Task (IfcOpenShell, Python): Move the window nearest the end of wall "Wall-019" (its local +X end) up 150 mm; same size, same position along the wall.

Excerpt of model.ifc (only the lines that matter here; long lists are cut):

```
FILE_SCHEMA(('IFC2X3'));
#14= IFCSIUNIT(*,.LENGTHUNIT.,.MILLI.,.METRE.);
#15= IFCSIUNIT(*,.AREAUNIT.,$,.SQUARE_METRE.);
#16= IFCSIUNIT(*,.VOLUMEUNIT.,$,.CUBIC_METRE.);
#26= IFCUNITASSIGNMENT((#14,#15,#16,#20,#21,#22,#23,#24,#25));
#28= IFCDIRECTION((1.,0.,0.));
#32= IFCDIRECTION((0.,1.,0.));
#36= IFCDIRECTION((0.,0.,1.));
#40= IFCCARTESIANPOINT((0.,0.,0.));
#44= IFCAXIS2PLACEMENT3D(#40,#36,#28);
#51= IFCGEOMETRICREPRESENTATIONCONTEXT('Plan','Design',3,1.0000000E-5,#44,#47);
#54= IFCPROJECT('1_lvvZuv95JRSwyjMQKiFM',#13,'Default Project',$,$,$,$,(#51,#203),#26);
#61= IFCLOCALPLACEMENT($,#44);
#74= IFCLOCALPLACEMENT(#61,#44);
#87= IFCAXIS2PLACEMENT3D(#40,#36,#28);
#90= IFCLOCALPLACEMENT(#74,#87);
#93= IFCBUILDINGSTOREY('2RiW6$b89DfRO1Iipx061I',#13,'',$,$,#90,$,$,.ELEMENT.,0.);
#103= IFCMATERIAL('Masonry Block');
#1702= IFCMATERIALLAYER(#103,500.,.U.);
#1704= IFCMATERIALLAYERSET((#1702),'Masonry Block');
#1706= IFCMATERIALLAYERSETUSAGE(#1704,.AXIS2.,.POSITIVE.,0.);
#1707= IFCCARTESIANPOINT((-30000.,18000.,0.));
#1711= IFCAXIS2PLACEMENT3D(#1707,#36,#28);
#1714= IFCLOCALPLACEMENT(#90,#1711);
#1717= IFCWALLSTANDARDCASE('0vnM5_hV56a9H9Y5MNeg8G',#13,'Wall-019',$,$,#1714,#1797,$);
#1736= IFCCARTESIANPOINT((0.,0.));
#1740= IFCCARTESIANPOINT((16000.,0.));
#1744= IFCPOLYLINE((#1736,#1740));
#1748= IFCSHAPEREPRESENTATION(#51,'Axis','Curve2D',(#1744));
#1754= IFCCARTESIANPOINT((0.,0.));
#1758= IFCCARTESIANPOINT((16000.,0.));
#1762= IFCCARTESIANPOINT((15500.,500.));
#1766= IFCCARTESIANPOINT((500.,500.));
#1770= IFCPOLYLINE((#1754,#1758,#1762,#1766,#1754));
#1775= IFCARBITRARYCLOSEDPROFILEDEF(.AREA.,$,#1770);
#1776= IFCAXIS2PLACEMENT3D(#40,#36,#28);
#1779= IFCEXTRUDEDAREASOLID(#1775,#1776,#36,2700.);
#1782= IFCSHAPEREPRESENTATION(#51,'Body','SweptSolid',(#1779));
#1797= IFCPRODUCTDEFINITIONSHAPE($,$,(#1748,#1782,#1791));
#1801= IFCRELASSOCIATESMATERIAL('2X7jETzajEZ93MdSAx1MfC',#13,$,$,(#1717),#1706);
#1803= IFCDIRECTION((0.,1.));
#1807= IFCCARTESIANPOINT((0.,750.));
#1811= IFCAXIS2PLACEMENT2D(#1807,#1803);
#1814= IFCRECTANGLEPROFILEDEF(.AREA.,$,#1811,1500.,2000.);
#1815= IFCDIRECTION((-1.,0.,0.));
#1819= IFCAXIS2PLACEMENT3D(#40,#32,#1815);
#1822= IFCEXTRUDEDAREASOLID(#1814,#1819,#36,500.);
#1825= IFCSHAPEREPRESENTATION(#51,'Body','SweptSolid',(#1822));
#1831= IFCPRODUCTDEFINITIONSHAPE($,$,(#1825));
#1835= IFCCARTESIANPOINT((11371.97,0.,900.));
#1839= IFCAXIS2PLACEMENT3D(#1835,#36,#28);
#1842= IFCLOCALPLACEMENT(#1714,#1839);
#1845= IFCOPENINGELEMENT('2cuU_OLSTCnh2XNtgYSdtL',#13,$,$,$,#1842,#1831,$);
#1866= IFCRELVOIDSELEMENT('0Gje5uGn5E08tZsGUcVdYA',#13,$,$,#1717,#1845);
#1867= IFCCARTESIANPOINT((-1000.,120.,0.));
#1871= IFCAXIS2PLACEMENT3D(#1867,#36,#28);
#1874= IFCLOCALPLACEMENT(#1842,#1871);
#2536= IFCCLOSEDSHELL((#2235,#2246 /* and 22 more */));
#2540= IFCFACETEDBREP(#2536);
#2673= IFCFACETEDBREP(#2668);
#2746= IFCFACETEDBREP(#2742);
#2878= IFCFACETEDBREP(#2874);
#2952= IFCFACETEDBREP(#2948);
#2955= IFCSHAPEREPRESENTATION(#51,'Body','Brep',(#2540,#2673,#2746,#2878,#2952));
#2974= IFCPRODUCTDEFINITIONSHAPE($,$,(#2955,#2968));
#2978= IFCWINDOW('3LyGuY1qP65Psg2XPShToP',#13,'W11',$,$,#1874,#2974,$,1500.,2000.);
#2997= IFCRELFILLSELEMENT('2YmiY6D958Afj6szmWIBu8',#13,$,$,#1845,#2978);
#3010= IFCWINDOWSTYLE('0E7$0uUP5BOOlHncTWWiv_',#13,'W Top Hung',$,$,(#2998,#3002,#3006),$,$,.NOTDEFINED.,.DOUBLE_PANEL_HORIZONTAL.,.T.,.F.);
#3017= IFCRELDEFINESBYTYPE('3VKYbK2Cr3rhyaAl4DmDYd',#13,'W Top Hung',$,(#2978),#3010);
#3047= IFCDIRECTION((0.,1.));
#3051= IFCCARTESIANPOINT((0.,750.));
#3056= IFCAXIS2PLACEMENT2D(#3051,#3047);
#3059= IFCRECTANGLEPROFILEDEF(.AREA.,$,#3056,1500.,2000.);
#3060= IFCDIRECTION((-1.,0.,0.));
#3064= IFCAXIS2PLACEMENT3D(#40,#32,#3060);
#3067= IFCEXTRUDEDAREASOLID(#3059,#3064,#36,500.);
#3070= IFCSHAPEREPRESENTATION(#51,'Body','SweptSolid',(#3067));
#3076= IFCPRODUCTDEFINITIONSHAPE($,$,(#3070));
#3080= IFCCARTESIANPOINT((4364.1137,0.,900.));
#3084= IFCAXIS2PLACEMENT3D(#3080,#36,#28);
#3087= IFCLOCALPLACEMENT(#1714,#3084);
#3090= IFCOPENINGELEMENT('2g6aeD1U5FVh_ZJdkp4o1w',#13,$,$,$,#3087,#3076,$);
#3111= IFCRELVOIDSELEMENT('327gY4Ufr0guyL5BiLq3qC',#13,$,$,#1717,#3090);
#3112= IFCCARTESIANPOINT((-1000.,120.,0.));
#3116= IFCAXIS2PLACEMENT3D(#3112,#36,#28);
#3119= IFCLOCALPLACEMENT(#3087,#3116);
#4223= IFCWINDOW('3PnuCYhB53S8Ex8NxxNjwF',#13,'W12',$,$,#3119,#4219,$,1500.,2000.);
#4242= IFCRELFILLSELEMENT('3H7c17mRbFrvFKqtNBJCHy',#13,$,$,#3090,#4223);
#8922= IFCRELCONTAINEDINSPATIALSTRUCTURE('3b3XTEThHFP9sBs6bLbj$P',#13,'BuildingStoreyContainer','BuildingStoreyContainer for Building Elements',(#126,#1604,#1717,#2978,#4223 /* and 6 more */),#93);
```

```python
import numpy as np
import ifcopenshell
import ifcopenshell.api.geometry
import ifcopenshell.util.placement
import ifcopenshell.util.unit

model = ifcopenshell.open("model.ifc")
unit_scale = ifcopenshell.util.unit.calculate_unit_scale(model)

window = model.by_guid("3LyGuY1qP65Psg2XPShToP")
opening = window.FillsVoids[0].RelatingOpeningElement
dz = 150.0

shift = np.array([0.0, 0.0, dz])
# The window is placed relative to its opening, so it follows when the opening moves.
matrix = ifcopenshell.util.placement.get_local_placement(opening.ObjectPlacement)
matrix[:3, 3] += shift
ifcopenshell.api.geometry.edit_object_placement(
    model, product=opening, matrix=matrix, is_si=False, should_transform_children=True
)

print(f"moved by {dz * unit_scale:+.3f} m")

model.write("model_updated.ifc")
```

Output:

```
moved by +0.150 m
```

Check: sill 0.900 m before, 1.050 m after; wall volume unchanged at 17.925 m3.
